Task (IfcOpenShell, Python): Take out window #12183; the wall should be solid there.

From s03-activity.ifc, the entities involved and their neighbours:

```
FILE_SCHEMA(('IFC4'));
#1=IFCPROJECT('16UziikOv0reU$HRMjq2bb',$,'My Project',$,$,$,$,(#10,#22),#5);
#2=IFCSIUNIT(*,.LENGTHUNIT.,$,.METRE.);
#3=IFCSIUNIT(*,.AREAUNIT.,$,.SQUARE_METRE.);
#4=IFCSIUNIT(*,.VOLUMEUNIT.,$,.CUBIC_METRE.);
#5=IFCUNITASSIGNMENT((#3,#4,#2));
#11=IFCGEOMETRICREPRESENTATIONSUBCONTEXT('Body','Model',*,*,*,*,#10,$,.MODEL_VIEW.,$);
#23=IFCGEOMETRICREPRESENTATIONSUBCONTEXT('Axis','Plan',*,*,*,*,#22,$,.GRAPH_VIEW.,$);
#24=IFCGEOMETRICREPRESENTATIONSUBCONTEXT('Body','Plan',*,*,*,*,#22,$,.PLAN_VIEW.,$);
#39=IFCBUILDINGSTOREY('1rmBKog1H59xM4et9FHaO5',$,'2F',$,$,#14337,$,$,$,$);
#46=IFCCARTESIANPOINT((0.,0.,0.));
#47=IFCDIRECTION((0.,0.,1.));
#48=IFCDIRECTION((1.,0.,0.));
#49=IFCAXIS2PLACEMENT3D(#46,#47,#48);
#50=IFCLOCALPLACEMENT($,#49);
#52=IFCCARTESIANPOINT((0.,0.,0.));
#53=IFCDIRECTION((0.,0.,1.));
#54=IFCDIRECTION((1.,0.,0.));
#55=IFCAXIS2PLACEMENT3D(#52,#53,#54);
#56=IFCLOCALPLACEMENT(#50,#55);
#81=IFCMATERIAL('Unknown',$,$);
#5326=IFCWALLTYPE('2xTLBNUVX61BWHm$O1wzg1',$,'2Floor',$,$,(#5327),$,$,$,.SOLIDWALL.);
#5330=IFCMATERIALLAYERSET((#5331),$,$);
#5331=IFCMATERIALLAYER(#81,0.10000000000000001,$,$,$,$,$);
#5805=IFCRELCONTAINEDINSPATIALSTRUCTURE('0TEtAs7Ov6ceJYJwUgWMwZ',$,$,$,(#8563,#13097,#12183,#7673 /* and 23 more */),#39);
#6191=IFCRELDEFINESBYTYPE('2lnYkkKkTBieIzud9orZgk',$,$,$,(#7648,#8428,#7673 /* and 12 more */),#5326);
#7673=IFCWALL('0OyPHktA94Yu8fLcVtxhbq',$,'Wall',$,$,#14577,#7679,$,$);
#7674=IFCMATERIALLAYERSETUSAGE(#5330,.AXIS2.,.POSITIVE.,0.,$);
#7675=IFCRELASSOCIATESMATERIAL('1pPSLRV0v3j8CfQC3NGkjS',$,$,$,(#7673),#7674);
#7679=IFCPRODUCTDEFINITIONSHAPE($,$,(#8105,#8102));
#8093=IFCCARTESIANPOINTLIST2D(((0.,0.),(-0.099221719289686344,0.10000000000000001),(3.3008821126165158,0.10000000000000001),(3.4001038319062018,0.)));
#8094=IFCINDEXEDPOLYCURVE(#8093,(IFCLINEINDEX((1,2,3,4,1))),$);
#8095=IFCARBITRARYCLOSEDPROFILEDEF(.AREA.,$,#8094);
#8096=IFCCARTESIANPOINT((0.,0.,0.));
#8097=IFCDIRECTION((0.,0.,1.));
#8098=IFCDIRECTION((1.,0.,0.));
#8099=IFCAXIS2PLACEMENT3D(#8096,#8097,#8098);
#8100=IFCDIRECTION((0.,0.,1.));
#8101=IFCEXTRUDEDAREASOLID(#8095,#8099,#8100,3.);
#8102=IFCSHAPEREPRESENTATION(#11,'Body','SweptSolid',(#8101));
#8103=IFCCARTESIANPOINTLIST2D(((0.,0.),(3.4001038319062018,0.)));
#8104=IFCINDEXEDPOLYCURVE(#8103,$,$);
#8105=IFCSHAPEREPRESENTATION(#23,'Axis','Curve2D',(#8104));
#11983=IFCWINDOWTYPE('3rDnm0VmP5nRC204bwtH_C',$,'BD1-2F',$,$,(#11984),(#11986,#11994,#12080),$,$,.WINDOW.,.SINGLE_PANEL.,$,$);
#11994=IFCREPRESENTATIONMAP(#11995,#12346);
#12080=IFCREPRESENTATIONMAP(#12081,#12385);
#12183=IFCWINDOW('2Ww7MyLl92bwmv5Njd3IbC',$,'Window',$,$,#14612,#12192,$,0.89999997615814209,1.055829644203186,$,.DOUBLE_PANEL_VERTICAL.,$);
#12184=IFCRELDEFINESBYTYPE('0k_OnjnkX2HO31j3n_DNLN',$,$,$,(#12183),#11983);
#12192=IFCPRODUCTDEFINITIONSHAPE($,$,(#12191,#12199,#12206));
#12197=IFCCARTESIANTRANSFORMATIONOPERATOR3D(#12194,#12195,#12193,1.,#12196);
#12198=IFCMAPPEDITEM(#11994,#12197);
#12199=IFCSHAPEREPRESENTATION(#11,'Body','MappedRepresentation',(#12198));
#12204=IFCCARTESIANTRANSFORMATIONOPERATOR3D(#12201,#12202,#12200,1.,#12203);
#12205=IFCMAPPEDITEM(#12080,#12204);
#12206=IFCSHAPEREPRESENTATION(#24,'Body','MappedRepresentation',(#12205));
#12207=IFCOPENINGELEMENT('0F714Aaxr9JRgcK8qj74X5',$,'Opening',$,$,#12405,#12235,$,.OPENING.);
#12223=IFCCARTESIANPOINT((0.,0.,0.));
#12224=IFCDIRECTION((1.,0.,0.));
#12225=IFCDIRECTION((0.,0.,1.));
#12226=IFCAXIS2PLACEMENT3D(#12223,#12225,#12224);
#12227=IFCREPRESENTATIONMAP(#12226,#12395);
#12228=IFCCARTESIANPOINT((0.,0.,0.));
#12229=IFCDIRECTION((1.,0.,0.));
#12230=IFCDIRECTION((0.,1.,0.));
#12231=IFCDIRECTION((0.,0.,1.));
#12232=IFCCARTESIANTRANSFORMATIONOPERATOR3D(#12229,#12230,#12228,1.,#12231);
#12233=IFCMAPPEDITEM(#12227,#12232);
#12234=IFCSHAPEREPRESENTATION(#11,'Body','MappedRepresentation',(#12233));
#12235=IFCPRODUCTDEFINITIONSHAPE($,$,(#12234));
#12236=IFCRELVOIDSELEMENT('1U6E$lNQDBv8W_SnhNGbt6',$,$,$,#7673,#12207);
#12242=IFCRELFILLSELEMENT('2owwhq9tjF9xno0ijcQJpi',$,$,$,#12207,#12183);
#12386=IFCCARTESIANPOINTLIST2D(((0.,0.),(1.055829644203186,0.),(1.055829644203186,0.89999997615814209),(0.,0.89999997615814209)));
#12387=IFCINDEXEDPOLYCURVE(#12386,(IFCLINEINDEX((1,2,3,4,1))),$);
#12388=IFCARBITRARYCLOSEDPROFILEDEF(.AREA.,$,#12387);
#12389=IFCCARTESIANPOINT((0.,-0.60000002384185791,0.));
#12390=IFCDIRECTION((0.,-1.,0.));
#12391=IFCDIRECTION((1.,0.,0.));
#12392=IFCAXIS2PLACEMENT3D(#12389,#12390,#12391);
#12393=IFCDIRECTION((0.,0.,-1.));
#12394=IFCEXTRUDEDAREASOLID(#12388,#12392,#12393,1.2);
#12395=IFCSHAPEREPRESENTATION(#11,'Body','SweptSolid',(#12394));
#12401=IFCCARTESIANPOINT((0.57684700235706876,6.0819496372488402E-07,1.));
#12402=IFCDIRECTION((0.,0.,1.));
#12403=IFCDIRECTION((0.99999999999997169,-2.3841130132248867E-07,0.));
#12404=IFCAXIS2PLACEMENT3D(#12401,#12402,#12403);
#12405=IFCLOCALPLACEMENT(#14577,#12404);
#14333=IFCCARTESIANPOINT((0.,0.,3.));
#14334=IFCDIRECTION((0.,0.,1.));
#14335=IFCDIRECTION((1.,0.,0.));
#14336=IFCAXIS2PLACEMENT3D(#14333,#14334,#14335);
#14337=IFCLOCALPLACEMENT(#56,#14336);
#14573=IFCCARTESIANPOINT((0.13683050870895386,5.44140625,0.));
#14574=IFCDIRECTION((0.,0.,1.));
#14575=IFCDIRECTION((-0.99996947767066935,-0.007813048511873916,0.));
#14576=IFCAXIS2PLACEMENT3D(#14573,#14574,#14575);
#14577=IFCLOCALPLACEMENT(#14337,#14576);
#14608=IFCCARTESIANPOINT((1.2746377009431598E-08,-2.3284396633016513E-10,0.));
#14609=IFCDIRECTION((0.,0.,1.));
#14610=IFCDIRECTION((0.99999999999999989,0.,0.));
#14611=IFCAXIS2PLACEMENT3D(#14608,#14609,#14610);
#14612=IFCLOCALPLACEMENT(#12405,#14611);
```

```python
import ifcopenshell
import ifcopenshell.api.feature
import ifcopenshell.api.root
import ifcopenshell.geom
import ifcopenshell.util.shape

model = ifcopenshell.open("s03-activity.ifc")
settings = ifcopenshell.geom.settings()


def volume(element):
    """Net volume in cubic metres, openings subtracted."""
    shape = ifcopenshell.geom.create_shape(settings, element)
    return ifcopenshell.util.shape.get_volume(shape.geometry)


window = model.by_guid("2Ww7MyLl92bwmv5Njd3IbC")
opening = window.FillsVoids[0].RelatingOpeningElement
wall = opening.VoidsElements[0].RelatingBuildingElement
before = volume(wall)

ifcopenshell.api.root.remove_product(model, product=window)
ifcopenshell.api.feature.remove_feature(model, feature=opening)

after = volume(wall)

print(f"wall volume {before:.3f} -> {after:.3f} m3")

model.write("s03-activity_v2.ifc")
```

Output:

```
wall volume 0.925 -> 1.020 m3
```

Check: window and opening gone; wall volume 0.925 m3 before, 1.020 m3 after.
